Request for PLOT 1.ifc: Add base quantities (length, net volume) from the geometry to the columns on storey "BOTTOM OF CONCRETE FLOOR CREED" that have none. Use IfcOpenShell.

First a look at what the model holds.

```python
import ifcopenshell
import ifcopenshell.util.element
import ifcopenshell.util.unit

model = ifcopenshell.open("PLOT 1.ifc")
print(model.schema)
for unit_type in ("LENGTHUNIT", "AREAUNIT", "VOLUMEUNIT"):
    print(unit_type, ifcopenshell.util.unit.calculate_unit_scale(model, unit_type))
storey = next(s for s in model.by_type("IfcBuildingStorey") if s.Name == "BOTTOM OF CONCRETE FLOOR CREED")
columns = [e for e in ifcopenshell.util.element.get_decomposition(storey) if e.is_a("IfcColumn")]
for e in sorted(columns, key=lambda e: e.id()):
    print(e.id(), e.is_a(), e.Name, list(ifcopenshell.util.element.get_psets(e, qtos_only=True)), sep=" | ")
```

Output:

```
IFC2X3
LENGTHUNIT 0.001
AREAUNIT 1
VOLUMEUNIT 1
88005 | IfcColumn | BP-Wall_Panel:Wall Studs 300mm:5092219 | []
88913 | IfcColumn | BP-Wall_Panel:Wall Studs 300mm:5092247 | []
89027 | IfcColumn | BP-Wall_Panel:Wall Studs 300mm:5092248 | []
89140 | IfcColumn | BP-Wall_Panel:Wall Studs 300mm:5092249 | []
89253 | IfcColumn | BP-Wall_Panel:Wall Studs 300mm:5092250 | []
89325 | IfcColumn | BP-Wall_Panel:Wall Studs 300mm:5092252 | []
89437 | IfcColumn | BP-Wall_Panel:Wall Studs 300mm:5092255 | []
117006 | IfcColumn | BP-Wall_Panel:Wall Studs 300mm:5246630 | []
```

```python
import ifcopenshell
import ifcopenshell.api.pset
import ifcopenshell.geom
import ifcopenshell.util.element
import ifcopenshell.util.shape
import ifcopenshell.util.unit

model = ifcopenshell.open("PLOT 1.ifc")
unit_scale = ifcopenshell.util.unit.calculate_unit_scale(model)
volume_scale = ifcopenshell.util.unit.calculate_unit_scale(model, "VOLUMEUNIT")
settings = ifcopenshell.geom.settings()

storey = next(s for s in model.by_type("IfcBuildingStorey") if s.Name == "BOTTOM OF CONCRETE FLOOR CREED")
columns = [e for e in ifcopenshell.util.element.get_decomposition(storey) if e.is_a("IfcColumn")]

for e in sorted(columns, key=lambda e: e.id()):
    if ifcopenshell.util.element.get_psets(e, qtos_only=True, should_inherit=False):
        continue
    # Geometry comes back in metres, in the element's own axes.
    shape = ifcopenshell.geom.create_shape(settings, e)
    values = {
        "Length": ifcopenshell.util.shape.get_z(shape.geometry) / unit_scale,
        "NetVolume": ifcopenshell.util.shape.get_volume(shape.geometry) / volume_scale,
    }
    qto = ifcopenshell.api.pset.add_qto(model, product=e, name="BaseQuantities")
    ifcopenshell.api.pset.edit_qto(model, qto=qto, properties=values)
    print(e.id(), {k: round(v, 3) for k, v in values.items()})

model.write("PLOT 1_updated.ifc")
```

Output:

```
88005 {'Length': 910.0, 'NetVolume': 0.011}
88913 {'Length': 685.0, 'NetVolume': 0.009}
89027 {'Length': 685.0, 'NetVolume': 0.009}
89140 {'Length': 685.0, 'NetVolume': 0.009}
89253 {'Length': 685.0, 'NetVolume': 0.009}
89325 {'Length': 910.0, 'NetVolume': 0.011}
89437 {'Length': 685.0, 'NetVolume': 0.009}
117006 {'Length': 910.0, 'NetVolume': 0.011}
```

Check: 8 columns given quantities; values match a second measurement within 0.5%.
